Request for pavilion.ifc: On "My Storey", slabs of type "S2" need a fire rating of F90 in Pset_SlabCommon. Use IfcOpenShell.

First a look at what the model holds.

```python
import ifcopenshell
import ifcopenshell.util.element

model = ifcopenshell.open("pavilion.ifc")
print(model.schema)
storey = next(s for s in model.by_type("IfcBuildingStorey") if s.Name == "My Storey")
slabs = [e for e in ifcopenshell.util.element.get_decomposition(storey) if e.is_a("IfcSlab")]
seen = {}
for e in slabs:
    element_type = ifcopenshell.util.element.get_type(e)
    key = (element_type.Name if element_type != e and element_type else None, ifcopenshell.util.element.get_pset(e, "Pset_SlabCommon", "FireRating"))
    seen[key] = seen.get(key, 0) + 1
for (name, value), count in sorted(seen.items(), key=str):
    print(count, "x", name, "|", value)
```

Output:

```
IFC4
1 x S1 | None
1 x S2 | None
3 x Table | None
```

```python
import ifcopenshell
import ifcopenshell.api.pset
import ifcopenshell.util.element

model = ifcopenshell.open("pavilion.ifc")

storey = next(s for s in model.by_type("IfcBuildingStorey") if s.Name == "My Storey")
slabs = [e for e in ifcopenshell.util.element.get_decomposition(storey) if e.is_a("IfcSlab")]

count = 0
for e in slabs:
    element_type = ifcopenshell.util.element.get_type(e)
    if element_type in (None, e) or element_type.Name != "S2":
        continue
    # add_pset returns the element's existing set when there is one.
    pset = ifcopenshell.api.pset.add_pset(model, product=e, name="Pset_SlabCommon")
    ifcopenshell.api.pset.edit_pset(model, pset=pset, properties={"FireRating": "F90"})
    count += 1

print(count, "slabs updated")

model.write("pavilion_rev.ifc")
```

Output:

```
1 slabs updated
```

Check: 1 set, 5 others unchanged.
